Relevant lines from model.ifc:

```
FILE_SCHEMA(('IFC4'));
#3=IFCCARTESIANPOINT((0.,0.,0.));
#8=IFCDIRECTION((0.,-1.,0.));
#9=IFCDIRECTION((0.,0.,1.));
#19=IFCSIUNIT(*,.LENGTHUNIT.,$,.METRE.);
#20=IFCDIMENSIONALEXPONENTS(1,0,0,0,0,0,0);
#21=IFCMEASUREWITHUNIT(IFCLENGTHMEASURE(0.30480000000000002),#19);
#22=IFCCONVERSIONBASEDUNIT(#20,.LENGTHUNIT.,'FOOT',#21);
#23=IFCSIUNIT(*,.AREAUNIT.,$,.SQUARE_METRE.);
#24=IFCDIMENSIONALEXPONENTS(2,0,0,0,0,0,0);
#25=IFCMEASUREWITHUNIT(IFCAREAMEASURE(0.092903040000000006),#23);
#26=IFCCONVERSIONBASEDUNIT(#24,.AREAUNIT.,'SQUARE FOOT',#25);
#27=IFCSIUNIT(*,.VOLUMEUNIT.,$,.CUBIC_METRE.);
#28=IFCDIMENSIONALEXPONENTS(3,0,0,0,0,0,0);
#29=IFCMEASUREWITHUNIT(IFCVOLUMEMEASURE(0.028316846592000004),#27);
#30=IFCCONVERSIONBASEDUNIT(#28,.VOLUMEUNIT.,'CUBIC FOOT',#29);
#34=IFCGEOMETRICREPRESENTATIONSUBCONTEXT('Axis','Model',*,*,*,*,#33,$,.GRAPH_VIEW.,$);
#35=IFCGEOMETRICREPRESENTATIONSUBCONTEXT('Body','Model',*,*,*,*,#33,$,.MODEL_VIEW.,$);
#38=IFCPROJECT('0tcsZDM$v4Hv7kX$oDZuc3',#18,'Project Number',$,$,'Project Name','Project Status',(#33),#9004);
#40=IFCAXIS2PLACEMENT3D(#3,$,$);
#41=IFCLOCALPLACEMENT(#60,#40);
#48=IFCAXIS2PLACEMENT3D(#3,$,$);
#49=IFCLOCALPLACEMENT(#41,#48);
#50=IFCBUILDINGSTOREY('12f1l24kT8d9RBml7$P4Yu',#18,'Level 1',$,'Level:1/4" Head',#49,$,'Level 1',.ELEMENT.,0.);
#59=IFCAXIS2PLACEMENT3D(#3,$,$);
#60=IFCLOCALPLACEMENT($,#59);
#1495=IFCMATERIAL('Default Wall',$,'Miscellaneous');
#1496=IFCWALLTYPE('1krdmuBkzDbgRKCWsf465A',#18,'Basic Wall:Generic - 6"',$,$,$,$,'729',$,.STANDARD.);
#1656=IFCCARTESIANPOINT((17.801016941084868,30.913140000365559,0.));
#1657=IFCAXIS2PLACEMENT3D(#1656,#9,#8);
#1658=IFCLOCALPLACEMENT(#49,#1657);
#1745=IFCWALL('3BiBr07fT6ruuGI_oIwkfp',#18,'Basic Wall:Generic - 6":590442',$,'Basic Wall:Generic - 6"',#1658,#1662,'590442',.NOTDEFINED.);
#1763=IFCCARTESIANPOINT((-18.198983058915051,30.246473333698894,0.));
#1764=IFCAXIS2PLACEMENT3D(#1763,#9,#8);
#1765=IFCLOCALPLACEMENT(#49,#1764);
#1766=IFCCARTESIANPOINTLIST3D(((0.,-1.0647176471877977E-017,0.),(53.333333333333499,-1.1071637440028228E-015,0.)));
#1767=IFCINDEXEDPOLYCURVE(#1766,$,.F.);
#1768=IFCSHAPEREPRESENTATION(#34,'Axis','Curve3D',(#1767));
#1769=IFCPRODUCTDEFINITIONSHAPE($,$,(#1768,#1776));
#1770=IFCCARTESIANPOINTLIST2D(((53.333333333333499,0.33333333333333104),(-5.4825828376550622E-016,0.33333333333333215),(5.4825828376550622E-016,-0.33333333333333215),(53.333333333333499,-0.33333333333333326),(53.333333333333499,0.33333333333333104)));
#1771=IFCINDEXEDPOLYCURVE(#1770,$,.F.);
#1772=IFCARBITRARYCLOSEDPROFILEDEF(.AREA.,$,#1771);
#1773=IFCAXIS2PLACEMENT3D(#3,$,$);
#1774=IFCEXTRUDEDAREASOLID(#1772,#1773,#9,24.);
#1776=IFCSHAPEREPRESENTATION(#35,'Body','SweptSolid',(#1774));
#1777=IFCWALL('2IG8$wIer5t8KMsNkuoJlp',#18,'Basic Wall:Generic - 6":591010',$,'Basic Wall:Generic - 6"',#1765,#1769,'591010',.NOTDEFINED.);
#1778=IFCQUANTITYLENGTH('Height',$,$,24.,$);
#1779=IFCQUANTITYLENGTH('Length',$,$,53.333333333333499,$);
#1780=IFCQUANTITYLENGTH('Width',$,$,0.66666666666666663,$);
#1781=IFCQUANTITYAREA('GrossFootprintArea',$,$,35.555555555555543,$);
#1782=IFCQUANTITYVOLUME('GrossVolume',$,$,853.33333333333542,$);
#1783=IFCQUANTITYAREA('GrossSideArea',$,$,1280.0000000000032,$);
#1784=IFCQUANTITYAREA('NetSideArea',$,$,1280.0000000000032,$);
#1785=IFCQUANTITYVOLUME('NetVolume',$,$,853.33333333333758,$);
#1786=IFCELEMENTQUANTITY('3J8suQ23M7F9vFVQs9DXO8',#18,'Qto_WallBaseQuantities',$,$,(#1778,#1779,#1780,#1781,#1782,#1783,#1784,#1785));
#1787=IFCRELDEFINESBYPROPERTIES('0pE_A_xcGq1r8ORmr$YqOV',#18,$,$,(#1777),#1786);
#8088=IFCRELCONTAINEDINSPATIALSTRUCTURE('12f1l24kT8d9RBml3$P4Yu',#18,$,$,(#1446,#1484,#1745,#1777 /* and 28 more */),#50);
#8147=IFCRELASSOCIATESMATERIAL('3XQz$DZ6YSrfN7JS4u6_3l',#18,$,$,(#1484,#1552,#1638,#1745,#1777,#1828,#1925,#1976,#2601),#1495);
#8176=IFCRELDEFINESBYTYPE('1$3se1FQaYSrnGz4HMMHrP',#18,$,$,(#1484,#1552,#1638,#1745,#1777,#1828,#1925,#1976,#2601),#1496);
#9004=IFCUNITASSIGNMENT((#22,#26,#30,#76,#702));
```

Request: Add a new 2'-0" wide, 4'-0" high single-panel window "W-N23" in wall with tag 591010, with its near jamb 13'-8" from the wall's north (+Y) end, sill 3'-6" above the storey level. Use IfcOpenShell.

```python
import numpy as np
import ifcopenshell
import ifcopenshell.api.feature
import ifcopenshell.api.geometry
import ifcopenshell.api.pset
import ifcopenshell.api.root
import ifcopenshell.api.spatial
import ifcopenshell.geom
import ifcopenshell.util.element
import ifcopenshell.util.placement
import ifcopenshell.util.representation
import ifcopenshell.util.shape
import ifcopenshell.util.unit

model = ifcopenshell.open("model.ifc")
unit_scale = ifcopenshell.util.unit.calculate_unit_scale(model)
area_scale = ifcopenshell.util.unit.calculate_unit_scale(model, "AREAUNIT")
volume_scale = ifcopenshell.util.unit.calculate_unit_scale(model, "VOLUMEUNIT")
settings = ifcopenshell.geom.settings()


def volume(element):
    """Net volume in cubic metres, openings subtracted."""
    shape = ifcopenshell.geom.create_shape(settings, element)
    return ifcopenshell.util.shape.get_volume(shape.geometry)


wall = model.by_guid("2IG8$wIer5t8KMsNkuoJlp")
storey = ifcopenshell.util.element.get_container(wall, ifc_class="IfcBuildingStorey")
context = ifcopenshell.util.representation.get_context(model, "Model", "Body", "MODEL_VIEW")
before = volume(wall)

width, height, from_end, sill = 0.6096, 1.2192, 4.1656, 1.0668  # metres

# The wall runs along its own X axis, and the end named is its -X end.
wall_shape = ifcopenshell.geom.create_shape(settings, wall)
x, y, z = ifcopenshell.util.shape.get_vertices(wall_shape.geometry).T
start = x.min() + from_end
face, thickness = float(y.min()), float(y.max() - y.min())
wall_matrix = ifcopenshell.util.placement.get_local_placement(wall.ObjectPlacement)
level = ifcopenshell.util.placement.get_local_placement(storey.ObjectPlacement)[2, 3]


def in_wall(x, y):
    """Placement at x, y metres in the wall's axes, at sill height."""
    matrix = wall_matrix.copy()
    matrix[:, 3] = wall_matrix @ np.array([x / unit_scale, y / unit_scale, 0.0, 1.0])
    matrix[2, 3] = level + sill / unit_scale
    return matrix


# Opening: a box that overshoots both wall faces by 50 mm.
opening = ifcopenshell.api.root.create_entity(model, ifc_class="IfcOpeningElement", predefined_type="OPENING")
box = ifcopenshell.api.geometry.add_wall_representation(
    model, context=context, length=width, height=height, thickness=thickness + 0.1
)
ifcopenshell.api.geometry.assign_representation(model, product=opening, representation=box)
ifcopenshell.api.geometry.edit_object_placement(model, product=opening, matrix=in_wall(start, face - 0.05), is_si=False)
ifcopenshell.api.feature.add_feature(model, feature=opening, element=wall)

window = ifcopenshell.api.root.create_entity(model, ifc_class="IfcWindow", name="W-N23", predefined_type="WINDOW")
window.OverallWidth, window.OverallHeight = width / unit_scale, height / unit_scale
window.PartitioningType = "SINGLE_PANEL"
body = ifcopenshell.api.geometry.add_window_representation(
    model,
    context=context,
    overall_width=window.OverallWidth,
    overall_height=window.OverallHeight,
    partition_type="SINGLE_PANEL",
)
ifcopenshell.api.geometry.assign_representation(model, product=window, representation=body)
ifcopenshell.api.spatial.assign_container(model, products=[window], relating_structure=storey)
ifcopenshell.api.feature.add_filling(model, opening=opening, element=window)

# Centre the window in the wall's thickness.
ifcopenshell.api.geometry.edit_object_placement(model, product=window, matrix=in_wall(start, face), is_si=False)
window_shape = ifcopenshell.geom.create_shape(settings, window)
depth = ifcopenshell.util.shape.get_vertices(window_shape.geometry)[:, 1]
offset = face + thickness / 2 - (depth.min() + depth.max()) / 2
ifcopenshell.api.geometry.edit_object_placement(model, product=window, matrix=in_wall(start, offset), is_si=False)

after = volume(wall)

# Update the wall's stored quantities.
qto = model.by_id(ifcopenshell.util.element.get_pset(wall, "Qto_WallBaseQuantities", should_inherit=False)["id"])
ifcopenshell.api.pset.edit_qto(model, qto=qto, properties={
    "NetSideArea": after / thickness / area_scale,
    "NetVolume": after / volume_scale,
})

print(f"wall volume {before:.3f} -> {after:.3f} m3")

model.write("model_rev.ifc")
```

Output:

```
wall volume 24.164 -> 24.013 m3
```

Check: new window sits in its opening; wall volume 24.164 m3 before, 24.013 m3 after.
